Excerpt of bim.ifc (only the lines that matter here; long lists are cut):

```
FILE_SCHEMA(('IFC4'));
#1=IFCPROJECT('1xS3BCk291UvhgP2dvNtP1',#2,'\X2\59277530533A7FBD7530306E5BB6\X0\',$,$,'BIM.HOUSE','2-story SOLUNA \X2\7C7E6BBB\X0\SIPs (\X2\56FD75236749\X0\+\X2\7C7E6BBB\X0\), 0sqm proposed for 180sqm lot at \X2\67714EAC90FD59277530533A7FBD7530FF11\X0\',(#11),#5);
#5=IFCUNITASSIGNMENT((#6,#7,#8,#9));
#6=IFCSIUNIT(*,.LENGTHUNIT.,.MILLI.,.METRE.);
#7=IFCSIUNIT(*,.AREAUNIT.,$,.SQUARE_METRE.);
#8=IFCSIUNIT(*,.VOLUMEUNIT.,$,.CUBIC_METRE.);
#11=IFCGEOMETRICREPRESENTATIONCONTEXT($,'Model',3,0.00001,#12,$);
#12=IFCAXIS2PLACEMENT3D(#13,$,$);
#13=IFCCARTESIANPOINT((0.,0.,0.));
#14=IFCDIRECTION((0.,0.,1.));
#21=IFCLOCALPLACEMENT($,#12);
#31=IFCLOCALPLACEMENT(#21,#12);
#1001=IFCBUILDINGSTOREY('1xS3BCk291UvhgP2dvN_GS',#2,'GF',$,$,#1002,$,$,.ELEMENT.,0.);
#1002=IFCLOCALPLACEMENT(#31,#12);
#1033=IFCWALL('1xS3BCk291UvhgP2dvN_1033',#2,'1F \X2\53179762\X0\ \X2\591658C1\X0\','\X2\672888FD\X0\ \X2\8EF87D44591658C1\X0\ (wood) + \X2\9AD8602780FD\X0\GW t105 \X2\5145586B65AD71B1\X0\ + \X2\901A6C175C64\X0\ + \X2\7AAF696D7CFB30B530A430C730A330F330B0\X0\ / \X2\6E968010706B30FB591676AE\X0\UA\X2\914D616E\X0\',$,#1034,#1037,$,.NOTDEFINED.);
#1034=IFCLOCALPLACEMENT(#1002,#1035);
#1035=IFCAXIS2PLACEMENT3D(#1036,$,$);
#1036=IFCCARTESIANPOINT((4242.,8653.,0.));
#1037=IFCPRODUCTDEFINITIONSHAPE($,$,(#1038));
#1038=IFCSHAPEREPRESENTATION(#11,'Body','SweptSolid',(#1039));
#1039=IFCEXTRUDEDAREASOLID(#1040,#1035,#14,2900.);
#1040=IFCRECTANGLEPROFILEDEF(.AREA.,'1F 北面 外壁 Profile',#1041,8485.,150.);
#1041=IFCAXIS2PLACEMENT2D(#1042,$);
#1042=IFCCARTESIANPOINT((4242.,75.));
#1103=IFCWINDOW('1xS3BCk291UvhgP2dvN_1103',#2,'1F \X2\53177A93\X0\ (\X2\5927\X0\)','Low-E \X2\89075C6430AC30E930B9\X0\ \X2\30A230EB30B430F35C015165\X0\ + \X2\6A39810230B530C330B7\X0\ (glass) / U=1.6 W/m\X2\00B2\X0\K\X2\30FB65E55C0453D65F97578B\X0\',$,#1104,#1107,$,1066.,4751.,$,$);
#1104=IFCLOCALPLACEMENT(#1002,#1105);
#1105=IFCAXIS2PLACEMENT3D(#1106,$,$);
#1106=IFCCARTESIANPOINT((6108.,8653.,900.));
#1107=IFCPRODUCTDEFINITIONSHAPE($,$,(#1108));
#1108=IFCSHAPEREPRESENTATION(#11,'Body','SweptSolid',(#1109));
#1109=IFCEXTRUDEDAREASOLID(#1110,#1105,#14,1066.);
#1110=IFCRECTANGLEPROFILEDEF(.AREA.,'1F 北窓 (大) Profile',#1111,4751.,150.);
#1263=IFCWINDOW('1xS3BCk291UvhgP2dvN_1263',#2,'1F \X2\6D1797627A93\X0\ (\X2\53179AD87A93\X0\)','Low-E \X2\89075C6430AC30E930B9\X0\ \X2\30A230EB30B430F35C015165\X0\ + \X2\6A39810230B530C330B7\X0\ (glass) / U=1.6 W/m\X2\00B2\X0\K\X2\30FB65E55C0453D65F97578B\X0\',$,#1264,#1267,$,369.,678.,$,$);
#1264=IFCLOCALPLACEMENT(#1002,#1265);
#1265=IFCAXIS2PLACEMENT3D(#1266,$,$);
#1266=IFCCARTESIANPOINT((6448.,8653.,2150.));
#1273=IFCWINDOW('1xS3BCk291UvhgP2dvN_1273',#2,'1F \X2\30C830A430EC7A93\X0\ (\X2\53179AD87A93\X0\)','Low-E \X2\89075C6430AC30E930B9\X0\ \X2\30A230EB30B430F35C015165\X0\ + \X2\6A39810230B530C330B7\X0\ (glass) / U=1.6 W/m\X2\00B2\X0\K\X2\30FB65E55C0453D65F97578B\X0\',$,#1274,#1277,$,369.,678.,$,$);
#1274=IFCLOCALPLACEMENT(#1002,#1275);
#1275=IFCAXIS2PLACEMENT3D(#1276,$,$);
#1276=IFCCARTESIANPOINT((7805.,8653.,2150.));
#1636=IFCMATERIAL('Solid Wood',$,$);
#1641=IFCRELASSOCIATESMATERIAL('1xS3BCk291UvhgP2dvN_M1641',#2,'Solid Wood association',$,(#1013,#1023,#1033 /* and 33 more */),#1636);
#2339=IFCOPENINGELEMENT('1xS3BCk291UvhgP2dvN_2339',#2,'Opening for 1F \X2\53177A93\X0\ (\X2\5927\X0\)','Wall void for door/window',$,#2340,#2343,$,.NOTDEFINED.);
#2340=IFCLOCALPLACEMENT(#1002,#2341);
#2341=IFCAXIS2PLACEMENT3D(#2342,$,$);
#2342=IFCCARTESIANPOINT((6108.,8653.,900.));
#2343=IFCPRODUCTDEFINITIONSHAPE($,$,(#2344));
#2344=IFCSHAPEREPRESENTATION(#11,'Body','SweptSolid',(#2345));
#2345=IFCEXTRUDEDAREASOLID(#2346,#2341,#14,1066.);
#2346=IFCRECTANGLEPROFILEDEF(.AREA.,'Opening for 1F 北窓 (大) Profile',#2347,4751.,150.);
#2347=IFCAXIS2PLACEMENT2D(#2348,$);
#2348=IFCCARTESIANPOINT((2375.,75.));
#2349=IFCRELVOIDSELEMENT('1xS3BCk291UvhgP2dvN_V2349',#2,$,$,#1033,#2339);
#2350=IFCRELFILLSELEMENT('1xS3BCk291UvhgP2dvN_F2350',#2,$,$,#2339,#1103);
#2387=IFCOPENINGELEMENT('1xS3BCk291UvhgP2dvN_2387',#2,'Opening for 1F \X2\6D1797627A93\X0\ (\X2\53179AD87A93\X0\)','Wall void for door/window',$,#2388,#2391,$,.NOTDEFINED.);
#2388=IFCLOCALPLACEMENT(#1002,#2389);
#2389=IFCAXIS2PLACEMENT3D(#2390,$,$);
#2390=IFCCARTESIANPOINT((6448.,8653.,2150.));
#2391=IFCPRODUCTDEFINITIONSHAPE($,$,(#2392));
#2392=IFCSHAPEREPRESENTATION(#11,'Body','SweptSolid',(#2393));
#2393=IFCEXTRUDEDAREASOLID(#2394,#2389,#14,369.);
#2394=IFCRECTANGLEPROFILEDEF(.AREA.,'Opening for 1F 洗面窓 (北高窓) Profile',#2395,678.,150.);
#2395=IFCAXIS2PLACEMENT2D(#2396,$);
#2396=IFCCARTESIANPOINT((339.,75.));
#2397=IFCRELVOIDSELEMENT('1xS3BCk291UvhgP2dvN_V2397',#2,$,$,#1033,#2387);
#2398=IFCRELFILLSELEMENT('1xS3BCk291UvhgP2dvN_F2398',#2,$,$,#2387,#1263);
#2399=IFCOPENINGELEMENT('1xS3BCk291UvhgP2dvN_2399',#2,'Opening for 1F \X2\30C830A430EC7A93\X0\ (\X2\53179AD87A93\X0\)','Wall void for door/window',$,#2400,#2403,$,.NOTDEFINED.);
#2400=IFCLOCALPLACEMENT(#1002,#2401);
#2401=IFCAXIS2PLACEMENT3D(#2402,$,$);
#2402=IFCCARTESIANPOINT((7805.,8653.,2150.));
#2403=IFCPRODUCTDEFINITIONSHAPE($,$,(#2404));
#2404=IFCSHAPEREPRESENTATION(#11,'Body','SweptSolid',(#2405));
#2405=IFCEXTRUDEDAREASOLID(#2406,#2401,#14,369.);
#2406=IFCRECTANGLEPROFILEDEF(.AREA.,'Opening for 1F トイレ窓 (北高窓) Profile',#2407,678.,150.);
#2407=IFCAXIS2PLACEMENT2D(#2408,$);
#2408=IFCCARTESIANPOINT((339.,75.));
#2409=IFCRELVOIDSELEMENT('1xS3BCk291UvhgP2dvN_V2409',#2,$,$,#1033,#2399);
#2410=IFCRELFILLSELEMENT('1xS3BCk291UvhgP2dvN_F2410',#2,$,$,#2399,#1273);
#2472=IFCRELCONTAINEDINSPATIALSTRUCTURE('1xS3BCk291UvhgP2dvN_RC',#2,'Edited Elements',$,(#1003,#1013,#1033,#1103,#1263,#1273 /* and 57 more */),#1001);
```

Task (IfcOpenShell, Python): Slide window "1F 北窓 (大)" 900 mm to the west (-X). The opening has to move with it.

```python
import ifcopenshell
import ifcopenshell.api.geometry
import ifcopenshell.util.placement
import ifcopenshell.util.unit

model = ifcopenshell.open("bim.ifc")
unit_scale = ifcopenshell.util.unit.calculate_unit_scale(model)

window = model.by_id(1103)
opening = window.FillsVoids[0].RelatingOpeningElement
wall = opening.VoidsElements[0].RelatingBuildingElement

wall_matrix = ifcopenshell.util.placement.get_local_placement(wall.ObjectPlacement)
shift = wall_matrix[:3, 0] * -0.9 / unit_scale
before = ifcopenshell.util.placement.get_local_placement(window.ObjectPlacement)[:3, 3].copy()

# The window is not placed relative to its opening, so move both.
for product in (opening, window):
    matrix = ifcopenshell.util.placement.get_local_placement(product.ObjectPlacement)
    matrix[:3, 3] += shift
    ifcopenshell.api.geometry.edit_object_placement(model, product=product, matrix=matrix, is_si=False)

after = ifcopenshell.util.placement.get_local_placement(window.ObjectPlacement)[:3, 3]
print("window moved by", (after - before).round(3) + 0.0)

model.write("bim-out.ifc")
```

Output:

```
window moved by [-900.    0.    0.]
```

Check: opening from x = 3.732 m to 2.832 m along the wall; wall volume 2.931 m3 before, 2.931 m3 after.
